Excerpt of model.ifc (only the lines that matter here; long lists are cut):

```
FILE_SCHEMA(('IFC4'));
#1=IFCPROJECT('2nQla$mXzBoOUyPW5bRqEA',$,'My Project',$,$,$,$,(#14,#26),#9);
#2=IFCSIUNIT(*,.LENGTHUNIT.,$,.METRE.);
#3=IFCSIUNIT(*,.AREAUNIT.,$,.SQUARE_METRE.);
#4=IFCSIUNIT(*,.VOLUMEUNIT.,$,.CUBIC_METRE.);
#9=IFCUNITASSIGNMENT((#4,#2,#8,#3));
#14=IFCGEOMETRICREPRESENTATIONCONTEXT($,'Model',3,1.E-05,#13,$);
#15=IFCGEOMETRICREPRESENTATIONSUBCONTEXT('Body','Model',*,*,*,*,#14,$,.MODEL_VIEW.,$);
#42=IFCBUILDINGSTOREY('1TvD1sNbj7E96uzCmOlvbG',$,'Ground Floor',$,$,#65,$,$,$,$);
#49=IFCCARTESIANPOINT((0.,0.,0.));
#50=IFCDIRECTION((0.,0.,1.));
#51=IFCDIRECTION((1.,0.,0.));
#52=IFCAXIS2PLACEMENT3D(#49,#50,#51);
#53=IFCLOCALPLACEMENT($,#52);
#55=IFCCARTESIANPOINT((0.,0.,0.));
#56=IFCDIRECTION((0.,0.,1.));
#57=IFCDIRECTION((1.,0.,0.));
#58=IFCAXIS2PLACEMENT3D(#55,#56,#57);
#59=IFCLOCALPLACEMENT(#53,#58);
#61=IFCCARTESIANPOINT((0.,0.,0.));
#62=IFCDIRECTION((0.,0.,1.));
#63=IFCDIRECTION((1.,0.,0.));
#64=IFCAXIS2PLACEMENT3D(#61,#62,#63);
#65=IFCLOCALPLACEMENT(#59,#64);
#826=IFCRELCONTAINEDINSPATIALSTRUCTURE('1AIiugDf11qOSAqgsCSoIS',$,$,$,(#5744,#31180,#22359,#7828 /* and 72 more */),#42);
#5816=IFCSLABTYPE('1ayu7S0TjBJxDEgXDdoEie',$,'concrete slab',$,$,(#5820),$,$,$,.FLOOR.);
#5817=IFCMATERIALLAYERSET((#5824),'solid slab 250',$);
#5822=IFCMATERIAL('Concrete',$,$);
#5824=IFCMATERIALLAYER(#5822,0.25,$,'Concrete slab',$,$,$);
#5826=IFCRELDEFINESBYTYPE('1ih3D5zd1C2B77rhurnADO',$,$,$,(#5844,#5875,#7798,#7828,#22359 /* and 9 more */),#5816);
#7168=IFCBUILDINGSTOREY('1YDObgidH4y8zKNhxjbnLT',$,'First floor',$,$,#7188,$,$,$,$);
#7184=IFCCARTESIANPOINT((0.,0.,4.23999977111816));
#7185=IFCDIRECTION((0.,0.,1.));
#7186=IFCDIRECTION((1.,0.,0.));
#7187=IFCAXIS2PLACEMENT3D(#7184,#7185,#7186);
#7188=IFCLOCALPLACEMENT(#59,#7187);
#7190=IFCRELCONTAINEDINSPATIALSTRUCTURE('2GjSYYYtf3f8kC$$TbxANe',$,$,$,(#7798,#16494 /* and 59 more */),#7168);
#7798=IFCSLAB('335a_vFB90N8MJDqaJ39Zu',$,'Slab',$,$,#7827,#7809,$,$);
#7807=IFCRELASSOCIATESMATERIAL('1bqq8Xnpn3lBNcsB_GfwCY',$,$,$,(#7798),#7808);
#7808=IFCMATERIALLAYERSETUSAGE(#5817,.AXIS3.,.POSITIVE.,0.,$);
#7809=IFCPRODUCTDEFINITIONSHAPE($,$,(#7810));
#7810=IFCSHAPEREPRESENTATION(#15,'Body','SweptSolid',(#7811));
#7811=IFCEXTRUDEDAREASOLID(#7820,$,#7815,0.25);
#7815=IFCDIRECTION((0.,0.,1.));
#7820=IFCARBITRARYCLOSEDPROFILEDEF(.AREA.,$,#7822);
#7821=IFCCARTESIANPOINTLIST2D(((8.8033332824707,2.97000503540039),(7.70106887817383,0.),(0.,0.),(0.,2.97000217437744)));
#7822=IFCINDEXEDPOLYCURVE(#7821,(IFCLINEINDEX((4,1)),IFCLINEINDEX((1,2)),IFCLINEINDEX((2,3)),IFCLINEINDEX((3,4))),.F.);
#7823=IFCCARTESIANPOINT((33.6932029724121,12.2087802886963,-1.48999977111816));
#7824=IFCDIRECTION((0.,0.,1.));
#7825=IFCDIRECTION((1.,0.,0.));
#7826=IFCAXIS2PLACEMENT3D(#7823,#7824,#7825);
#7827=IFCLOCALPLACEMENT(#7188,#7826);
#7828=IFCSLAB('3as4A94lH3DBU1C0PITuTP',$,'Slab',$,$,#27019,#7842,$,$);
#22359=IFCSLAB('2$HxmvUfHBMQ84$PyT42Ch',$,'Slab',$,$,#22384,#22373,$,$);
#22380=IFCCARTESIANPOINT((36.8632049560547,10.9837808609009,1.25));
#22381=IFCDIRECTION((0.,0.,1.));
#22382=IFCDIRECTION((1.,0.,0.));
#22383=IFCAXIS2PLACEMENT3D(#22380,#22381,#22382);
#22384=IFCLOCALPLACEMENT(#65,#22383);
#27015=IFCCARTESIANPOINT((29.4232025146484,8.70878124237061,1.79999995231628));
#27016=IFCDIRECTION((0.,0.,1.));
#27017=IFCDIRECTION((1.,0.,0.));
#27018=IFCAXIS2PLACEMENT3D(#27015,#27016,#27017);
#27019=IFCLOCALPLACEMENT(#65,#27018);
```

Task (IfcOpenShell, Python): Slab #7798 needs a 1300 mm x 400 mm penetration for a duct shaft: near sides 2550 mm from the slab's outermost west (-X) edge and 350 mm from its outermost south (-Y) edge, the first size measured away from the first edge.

```python
import numpy as np
import ifcopenshell
import ifcopenshell.api.feature
import ifcopenshell.api.geometry
import ifcopenshell.api.root
import ifcopenshell.geom
import ifcopenshell.util.placement
import ifcopenshell.util.representation
import ifcopenshell.util.shape
import ifcopenshell.util.unit

model = ifcopenshell.open("model.ifc")
unit_scale = ifcopenshell.util.unit.calculate_unit_scale(model)
settings = ifcopenshell.geom.settings()


def volume(element):
    """Net volume in cubic metres, openings subtracted."""
    shape = ifcopenshell.geom.create_shape(settings, element)
    return ifcopenshell.util.shape.get_volume(shape.geometry)


slab = model.by_guid("335a_vFB90N8MJDqaJ39Zu")
before = volume(slab)

# Extent in the slab's own axes, in metres. The edges named are its -X and -Y sides.
slab_shape = ifcopenshell.geom.create_shape(settings, slab)
vertices = ifcopenshell.util.shape.get_vertices(slab_shape.geometry)
x_min, y_min, bottom = vertices.min(axis=0)
top = vertices[:, 2].max()

opening = ifcopenshell.api.root.create_entity(model, ifc_class="IfcOpeningElement", name="Duct shaft opening", predefined_type="OPENING")
context = ifcopenshell.util.representation.get_context(model, "Model", "Body", "MODEL_VIEW")
width, depth = 1.3, 0.4
outline = [(0.0, 0.0), (width, 0.0), (width, depth), (0.0, depth), (0.0, 0.0)]
# Overshoot both faces by 50 mm so the cut is clean.
shape = ifcopenshell.api.geometry.add_slab_representation(
    model, context=context, depth=top - bottom + 0.1, polyline=outline
)
ifcopenshell.api.geometry.assign_representation(model, product=opening, representation=shape)

matrix = ifcopenshell.util.placement.get_local_placement(slab.ObjectPlacement)
matrix[:, 3] = matrix @ np.append(np.array([x_min + 2.55, y_min + 0.35, bottom - 0.05]) / unit_scale, 1.0)
ifcopenshell.api.geometry.edit_object_placement(model, product=opening, matrix=matrix, is_si=False)
ifcopenshell.api.feature.add_feature(model, feature=opening, element=slab)

after = volume(slab)

print(f"slab volume {before:.3f} -> {after:.3f} m3")

model.write("model-out.ifc")
```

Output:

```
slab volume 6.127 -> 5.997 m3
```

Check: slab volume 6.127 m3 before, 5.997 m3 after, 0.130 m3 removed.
